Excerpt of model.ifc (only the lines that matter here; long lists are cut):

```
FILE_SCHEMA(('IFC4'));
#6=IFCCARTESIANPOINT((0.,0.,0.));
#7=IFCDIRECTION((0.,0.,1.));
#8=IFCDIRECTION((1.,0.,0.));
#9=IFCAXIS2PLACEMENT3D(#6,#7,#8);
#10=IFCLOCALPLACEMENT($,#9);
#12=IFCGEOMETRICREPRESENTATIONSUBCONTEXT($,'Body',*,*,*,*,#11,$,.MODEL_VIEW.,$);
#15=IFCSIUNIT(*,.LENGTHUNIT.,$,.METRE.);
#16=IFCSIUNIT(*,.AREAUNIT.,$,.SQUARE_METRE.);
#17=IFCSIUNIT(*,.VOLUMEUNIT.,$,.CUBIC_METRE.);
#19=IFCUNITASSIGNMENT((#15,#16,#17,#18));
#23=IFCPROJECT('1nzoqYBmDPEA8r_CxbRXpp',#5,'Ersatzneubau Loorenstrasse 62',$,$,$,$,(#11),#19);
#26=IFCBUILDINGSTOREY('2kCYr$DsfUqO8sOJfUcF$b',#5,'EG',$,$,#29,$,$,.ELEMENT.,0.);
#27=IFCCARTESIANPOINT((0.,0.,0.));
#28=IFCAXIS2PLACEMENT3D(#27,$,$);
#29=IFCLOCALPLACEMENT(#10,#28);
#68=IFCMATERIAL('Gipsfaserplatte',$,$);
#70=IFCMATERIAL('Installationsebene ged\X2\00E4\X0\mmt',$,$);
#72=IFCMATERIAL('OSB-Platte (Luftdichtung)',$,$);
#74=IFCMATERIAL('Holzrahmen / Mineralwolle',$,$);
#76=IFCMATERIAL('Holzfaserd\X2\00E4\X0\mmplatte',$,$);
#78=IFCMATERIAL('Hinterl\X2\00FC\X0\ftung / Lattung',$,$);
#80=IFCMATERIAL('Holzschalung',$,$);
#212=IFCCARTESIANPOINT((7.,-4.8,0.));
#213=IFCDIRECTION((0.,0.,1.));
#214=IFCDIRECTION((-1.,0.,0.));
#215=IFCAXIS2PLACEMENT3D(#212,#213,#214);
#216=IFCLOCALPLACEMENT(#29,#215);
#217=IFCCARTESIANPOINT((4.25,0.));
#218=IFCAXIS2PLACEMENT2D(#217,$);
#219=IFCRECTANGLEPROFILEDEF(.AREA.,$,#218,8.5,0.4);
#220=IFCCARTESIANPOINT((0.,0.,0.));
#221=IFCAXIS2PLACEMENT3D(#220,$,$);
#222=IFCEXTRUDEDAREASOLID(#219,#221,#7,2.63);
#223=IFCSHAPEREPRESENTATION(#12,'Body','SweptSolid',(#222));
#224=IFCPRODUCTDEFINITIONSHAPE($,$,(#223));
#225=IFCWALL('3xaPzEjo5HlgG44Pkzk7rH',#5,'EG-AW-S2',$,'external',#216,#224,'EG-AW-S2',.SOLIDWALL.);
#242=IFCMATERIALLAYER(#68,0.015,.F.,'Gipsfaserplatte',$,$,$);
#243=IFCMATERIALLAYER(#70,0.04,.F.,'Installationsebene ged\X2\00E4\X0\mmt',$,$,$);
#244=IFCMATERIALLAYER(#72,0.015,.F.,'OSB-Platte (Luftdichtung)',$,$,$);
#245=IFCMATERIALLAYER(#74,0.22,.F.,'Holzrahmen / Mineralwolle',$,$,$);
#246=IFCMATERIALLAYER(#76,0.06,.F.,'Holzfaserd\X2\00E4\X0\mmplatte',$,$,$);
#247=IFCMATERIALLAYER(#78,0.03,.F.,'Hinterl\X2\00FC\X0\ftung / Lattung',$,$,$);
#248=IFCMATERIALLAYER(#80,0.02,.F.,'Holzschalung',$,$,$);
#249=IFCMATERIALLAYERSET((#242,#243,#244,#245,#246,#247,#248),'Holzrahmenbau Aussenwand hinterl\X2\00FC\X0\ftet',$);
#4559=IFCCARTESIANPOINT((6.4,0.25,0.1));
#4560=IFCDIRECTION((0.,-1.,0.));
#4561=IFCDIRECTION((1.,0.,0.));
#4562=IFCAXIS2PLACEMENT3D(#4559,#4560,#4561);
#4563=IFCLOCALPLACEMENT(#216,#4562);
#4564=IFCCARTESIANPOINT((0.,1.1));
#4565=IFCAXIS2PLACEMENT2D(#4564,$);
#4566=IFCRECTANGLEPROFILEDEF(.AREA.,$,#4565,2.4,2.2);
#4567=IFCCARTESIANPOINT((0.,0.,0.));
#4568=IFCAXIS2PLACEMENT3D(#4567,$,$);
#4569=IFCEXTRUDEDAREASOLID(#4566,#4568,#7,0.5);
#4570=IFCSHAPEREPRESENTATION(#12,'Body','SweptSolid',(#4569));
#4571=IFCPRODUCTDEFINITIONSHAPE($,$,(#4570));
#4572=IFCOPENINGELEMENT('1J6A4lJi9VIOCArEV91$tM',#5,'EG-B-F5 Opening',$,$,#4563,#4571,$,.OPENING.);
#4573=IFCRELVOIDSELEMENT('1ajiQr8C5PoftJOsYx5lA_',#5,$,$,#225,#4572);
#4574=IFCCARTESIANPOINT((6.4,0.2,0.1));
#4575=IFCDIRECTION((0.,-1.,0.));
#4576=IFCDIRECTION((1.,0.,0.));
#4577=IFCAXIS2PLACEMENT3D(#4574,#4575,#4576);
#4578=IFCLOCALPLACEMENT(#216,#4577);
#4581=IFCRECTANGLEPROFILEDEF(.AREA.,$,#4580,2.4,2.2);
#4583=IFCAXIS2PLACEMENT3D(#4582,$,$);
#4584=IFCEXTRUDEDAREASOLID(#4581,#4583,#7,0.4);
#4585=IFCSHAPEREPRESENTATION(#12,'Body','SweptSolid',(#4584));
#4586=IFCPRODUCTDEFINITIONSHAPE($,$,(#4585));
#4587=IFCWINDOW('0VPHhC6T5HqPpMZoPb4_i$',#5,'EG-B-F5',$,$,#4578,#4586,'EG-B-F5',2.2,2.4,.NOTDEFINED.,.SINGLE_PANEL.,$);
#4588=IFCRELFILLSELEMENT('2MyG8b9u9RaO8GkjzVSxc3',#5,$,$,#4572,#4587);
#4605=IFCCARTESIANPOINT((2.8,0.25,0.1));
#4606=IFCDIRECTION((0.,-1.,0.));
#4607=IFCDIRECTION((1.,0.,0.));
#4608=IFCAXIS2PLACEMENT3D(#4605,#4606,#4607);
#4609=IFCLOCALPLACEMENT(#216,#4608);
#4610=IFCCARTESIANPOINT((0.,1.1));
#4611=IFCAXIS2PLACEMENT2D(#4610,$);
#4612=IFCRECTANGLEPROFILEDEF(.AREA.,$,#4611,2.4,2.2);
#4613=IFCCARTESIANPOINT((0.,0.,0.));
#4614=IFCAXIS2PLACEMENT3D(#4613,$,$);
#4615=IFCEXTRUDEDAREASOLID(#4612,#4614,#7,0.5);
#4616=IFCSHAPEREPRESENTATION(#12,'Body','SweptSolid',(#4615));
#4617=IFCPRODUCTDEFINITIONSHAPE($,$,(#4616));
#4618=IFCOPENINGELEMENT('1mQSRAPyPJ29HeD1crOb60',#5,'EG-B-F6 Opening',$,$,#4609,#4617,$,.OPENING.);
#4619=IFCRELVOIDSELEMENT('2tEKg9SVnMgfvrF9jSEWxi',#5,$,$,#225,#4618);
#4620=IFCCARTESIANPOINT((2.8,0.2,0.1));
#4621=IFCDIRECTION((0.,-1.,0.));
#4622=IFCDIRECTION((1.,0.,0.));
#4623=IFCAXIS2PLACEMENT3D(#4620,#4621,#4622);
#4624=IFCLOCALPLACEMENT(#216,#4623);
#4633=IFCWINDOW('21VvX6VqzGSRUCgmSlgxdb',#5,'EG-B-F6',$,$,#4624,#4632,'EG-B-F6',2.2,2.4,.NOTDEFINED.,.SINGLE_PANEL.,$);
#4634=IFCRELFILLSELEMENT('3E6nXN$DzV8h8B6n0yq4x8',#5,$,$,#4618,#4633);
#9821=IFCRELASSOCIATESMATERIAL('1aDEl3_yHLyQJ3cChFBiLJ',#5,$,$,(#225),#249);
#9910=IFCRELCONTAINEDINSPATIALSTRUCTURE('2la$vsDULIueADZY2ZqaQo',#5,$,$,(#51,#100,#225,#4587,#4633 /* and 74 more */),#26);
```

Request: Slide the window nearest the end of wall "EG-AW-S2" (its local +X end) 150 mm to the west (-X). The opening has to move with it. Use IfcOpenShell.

```python
import ifcopenshell
import ifcopenshell.api.geometry
import ifcopenshell.util.placement

model = ifcopenshell.open("model.ifc")

window = model.by_id(4587)
opening = window.FillsVoids[0].RelatingOpeningElement
wall = opening.VoidsElements[0].RelatingBuildingElement

wall_matrix = ifcopenshell.util.placement.get_local_placement(wall.ObjectPlacement)
shift = wall_matrix[:3, 0] * 0.15
before = ifcopenshell.util.placement.get_local_placement(window.ObjectPlacement)[:3, 3].copy()

# The window is not placed relative to its opening, so move both.
for product in (opening, window):
    matrix = ifcopenshell.util.placement.get_local_placement(product.ObjectPlacement)
    matrix[:3, 3] += shift
    ifcopenshell.api.geometry.edit_object_placement(model, product=product, matrix=matrix, is_si=False)

after = ifcopenshell.util.placement.get_local_placement(window.ObjectPlacement)[:3, 3]
print("window moved by", (after - before).round(3) + 0.0)

model.write("model_rev.ifc")
```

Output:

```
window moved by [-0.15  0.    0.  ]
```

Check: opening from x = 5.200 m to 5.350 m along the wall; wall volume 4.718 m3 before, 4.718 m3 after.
